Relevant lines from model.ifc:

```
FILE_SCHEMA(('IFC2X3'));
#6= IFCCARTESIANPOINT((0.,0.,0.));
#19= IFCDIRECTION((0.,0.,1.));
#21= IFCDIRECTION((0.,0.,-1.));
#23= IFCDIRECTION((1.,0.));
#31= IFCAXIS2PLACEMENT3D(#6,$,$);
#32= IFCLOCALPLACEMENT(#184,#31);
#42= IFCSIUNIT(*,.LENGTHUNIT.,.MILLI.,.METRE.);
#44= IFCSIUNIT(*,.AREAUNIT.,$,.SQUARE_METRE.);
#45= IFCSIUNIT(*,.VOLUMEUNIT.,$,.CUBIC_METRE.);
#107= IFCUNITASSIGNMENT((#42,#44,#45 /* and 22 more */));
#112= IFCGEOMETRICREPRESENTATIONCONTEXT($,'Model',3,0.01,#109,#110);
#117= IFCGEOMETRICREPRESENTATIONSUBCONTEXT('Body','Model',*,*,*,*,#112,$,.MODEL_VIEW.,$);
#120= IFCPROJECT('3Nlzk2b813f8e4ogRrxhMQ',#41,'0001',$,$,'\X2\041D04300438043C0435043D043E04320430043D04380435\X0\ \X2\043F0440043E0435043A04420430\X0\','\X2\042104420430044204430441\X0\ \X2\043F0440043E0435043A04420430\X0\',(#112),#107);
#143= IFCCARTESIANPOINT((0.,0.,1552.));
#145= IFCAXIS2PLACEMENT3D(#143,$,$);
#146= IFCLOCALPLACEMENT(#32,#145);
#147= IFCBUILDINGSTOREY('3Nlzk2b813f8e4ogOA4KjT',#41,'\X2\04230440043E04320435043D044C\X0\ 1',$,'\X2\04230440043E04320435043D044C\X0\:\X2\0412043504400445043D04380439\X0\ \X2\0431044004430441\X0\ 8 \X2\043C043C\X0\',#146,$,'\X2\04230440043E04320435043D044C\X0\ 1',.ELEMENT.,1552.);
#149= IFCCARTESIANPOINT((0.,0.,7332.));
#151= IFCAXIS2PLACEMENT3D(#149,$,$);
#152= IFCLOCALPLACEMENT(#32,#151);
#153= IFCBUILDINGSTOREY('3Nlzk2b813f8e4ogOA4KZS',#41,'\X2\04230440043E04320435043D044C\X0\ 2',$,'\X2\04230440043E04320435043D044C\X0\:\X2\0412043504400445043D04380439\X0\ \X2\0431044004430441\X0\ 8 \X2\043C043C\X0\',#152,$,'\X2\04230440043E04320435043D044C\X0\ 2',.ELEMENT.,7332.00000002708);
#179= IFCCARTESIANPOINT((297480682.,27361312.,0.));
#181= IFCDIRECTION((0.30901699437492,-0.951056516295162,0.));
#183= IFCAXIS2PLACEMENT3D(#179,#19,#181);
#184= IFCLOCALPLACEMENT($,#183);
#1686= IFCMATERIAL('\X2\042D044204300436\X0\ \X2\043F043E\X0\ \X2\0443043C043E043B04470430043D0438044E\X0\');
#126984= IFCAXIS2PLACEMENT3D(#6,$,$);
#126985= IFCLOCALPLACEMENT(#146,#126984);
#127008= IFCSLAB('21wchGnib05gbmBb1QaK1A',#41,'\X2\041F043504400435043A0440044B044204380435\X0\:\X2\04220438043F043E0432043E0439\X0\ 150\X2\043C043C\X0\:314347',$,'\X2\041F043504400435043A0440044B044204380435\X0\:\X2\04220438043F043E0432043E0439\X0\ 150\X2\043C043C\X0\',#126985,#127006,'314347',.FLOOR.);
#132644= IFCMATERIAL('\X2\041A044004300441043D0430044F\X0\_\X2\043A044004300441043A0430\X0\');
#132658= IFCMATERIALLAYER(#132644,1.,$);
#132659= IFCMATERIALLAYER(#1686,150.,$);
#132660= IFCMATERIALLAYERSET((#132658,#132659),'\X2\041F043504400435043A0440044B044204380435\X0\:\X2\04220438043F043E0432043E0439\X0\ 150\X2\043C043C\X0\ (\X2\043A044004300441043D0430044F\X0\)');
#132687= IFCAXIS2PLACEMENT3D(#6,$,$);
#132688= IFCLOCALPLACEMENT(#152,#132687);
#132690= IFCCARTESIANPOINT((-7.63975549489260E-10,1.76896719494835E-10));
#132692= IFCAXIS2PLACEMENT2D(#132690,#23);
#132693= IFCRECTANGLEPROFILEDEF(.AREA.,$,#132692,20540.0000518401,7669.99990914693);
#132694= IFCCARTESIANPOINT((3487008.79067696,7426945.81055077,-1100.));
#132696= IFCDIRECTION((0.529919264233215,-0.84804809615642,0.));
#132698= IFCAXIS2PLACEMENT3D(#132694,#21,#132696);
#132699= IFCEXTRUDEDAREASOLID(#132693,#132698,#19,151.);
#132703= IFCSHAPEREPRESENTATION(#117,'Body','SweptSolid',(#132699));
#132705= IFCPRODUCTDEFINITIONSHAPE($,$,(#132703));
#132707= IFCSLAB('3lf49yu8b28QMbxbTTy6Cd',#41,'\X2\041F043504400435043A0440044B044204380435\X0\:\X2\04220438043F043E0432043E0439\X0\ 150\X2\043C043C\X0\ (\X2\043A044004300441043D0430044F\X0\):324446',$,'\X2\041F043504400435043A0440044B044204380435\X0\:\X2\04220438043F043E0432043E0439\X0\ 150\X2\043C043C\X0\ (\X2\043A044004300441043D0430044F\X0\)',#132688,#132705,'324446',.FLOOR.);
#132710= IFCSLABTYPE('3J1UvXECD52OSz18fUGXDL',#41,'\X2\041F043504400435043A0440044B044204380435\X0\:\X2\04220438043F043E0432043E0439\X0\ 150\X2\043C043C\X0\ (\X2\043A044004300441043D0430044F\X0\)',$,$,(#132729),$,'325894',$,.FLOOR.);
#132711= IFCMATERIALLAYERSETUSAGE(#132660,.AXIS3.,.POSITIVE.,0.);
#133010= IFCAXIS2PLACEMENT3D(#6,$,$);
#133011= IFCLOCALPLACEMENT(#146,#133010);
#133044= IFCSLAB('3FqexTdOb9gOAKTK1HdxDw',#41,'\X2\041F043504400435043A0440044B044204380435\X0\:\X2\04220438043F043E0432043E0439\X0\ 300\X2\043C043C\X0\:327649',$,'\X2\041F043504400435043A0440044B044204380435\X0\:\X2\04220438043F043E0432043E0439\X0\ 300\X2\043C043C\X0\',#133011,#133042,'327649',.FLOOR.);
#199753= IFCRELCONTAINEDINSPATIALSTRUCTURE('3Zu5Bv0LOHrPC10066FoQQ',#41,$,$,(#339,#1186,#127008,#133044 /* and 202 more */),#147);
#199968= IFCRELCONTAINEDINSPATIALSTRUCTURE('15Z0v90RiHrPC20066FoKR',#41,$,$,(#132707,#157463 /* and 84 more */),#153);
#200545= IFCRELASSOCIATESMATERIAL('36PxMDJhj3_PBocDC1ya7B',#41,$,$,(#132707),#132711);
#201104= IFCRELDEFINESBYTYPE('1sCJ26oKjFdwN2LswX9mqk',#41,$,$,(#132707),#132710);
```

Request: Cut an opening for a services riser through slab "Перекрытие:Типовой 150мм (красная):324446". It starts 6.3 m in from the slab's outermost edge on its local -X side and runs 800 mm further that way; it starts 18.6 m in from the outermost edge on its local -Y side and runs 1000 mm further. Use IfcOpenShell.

```python
import numpy as np
import ifcopenshell
import ifcopenshell.api.feature
import ifcopenshell.api.geometry
import ifcopenshell.api.root
import ifcopenshell.geom
import ifcopenshell.util.placement
import ifcopenshell.util.representation
import ifcopenshell.util.shape
import ifcopenshell.util.unit

model = ifcopenshell.open("model.ifc")
unit_scale = ifcopenshell.util.unit.calculate_unit_scale(model)
settings = ifcopenshell.geom.settings()


def volume(element):
    """Net volume in cubic metres, openings subtracted."""
    shape = ifcopenshell.geom.create_shape(settings, element)
    return ifcopenshell.util.shape.get_volume(shape.geometry)


slab = model.by_id(132707)
before = volume(slab)

# Extent in the slab's own axes, in metres. The edges named are its -X and -Y sides.
slab_shape = ifcopenshell.geom.create_shape(settings, slab)
vertices = ifcopenshell.util.shape.get_vertices(slab_shape.geometry)
x_min, y_min, bottom = vertices.min(axis=0)
top = vertices[:, 2].max()

opening = ifcopenshell.api.root.create_entity(model, ifc_class="IfcOpeningElement", name="Services riser opening")
context = ifcopenshell.util.representation.get_context(model, "Model", "Body", "MODEL_VIEW")
width, depth = 0.8, 1
outline = [(0.0, 0.0), (width, 0.0), (width, depth), (0.0, depth), (0.0, 0.0)]
# Overshoot both faces by 50 mm so the cut is clean.
shape = ifcopenshell.api.geometry.add_slab_representation(
    model, context=context, depth=top - bottom + 0.1, polyline=outline
)
ifcopenshell.api.geometry.assign_representation(model, product=opening, representation=shape)

matrix = ifcopenshell.util.placement.get_local_placement(slab.ObjectPlacement)
matrix[:, 3] = matrix @ np.append(np.array([x_min + 6.3, y_min + 18.6, bottom - 0.05]) / unit_scale, 1.0)
ifcopenshell.api.geometry.edit_object_placement(model, product=opening, matrix=matrix, is_si=False)
ifcopenshell.api.feature.add_feature(model, feature=opening, element=slab)

after = volume(slab)

print(f"slab volume {before:.3f} -> {after:.3f} m3")

model.write("model_v2.ifc")
```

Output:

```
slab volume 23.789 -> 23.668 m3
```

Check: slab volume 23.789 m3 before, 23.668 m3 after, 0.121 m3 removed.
